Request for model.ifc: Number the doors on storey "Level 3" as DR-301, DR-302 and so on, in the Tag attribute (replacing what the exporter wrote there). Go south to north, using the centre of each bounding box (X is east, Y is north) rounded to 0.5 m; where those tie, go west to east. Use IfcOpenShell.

First a look at what the model holds.

```python
import ifcopenshell
import ifcopenshell.util.element
import ifcopenshell.util.placement

model = ifcopenshell.open("model.ifc")
print(model.schema)
storey = next(s for s in model.by_type("IfcBuildingStorey") if s.Name == "Level 3")
doors = [e for e in ifcopenshell.util.element.get_decomposition(storey) if e.is_a("IfcDoor")]
for e in sorted(doors, key=lambda e: e.id()):
    origin = ifcopenshell.util.placement.get_local_placement(e.ObjectPlacement)[:3, 3]
    print(e.id(), e.Tag, e.Name, origin.round(2) + 0.0, sep=" | ")
```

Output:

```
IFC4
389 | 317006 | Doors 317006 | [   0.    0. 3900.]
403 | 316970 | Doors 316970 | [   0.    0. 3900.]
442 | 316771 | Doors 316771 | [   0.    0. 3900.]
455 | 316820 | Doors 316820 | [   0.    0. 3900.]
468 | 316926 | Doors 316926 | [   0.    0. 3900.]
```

```python
import ifcopenshell
import ifcopenshell.geom
import ifcopenshell.util.element
import ifcopenshell.util.shape

model = ifcopenshell.open("model.ifc")
settings = ifcopenshell.geom.settings()
settings.set("use-world-coords", True)


def centre(element):
    shape = ifcopenshell.geom.create_shape(settings, element)
    return ifcopenshell.util.shape.get_bbox_centroid(shape.geometry)


storey = next(s for s in model.by_type("IfcBuildingStorey") if s.Name == "Level 3")
doors = [e for e in ifcopenshell.util.element.get_decomposition(storey) if e.is_a("IfcDoor")]

# Insertion points can sit at a corner or the storey origin, so sort by the geometry (in metres).
centres = {e: centre(e) for e in doors}
doors.sort(key=lambda e: (round(centres[e][1] / 0.5), centres[e][0]))

for i, e in enumerate(doors, start=1):
    number = f"DR-3{i:02d}"
    e.Tag = number
    print(e.id(), number)

model.write("model_v2.ifc")
```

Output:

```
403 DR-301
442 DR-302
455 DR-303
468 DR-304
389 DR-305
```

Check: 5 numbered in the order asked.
